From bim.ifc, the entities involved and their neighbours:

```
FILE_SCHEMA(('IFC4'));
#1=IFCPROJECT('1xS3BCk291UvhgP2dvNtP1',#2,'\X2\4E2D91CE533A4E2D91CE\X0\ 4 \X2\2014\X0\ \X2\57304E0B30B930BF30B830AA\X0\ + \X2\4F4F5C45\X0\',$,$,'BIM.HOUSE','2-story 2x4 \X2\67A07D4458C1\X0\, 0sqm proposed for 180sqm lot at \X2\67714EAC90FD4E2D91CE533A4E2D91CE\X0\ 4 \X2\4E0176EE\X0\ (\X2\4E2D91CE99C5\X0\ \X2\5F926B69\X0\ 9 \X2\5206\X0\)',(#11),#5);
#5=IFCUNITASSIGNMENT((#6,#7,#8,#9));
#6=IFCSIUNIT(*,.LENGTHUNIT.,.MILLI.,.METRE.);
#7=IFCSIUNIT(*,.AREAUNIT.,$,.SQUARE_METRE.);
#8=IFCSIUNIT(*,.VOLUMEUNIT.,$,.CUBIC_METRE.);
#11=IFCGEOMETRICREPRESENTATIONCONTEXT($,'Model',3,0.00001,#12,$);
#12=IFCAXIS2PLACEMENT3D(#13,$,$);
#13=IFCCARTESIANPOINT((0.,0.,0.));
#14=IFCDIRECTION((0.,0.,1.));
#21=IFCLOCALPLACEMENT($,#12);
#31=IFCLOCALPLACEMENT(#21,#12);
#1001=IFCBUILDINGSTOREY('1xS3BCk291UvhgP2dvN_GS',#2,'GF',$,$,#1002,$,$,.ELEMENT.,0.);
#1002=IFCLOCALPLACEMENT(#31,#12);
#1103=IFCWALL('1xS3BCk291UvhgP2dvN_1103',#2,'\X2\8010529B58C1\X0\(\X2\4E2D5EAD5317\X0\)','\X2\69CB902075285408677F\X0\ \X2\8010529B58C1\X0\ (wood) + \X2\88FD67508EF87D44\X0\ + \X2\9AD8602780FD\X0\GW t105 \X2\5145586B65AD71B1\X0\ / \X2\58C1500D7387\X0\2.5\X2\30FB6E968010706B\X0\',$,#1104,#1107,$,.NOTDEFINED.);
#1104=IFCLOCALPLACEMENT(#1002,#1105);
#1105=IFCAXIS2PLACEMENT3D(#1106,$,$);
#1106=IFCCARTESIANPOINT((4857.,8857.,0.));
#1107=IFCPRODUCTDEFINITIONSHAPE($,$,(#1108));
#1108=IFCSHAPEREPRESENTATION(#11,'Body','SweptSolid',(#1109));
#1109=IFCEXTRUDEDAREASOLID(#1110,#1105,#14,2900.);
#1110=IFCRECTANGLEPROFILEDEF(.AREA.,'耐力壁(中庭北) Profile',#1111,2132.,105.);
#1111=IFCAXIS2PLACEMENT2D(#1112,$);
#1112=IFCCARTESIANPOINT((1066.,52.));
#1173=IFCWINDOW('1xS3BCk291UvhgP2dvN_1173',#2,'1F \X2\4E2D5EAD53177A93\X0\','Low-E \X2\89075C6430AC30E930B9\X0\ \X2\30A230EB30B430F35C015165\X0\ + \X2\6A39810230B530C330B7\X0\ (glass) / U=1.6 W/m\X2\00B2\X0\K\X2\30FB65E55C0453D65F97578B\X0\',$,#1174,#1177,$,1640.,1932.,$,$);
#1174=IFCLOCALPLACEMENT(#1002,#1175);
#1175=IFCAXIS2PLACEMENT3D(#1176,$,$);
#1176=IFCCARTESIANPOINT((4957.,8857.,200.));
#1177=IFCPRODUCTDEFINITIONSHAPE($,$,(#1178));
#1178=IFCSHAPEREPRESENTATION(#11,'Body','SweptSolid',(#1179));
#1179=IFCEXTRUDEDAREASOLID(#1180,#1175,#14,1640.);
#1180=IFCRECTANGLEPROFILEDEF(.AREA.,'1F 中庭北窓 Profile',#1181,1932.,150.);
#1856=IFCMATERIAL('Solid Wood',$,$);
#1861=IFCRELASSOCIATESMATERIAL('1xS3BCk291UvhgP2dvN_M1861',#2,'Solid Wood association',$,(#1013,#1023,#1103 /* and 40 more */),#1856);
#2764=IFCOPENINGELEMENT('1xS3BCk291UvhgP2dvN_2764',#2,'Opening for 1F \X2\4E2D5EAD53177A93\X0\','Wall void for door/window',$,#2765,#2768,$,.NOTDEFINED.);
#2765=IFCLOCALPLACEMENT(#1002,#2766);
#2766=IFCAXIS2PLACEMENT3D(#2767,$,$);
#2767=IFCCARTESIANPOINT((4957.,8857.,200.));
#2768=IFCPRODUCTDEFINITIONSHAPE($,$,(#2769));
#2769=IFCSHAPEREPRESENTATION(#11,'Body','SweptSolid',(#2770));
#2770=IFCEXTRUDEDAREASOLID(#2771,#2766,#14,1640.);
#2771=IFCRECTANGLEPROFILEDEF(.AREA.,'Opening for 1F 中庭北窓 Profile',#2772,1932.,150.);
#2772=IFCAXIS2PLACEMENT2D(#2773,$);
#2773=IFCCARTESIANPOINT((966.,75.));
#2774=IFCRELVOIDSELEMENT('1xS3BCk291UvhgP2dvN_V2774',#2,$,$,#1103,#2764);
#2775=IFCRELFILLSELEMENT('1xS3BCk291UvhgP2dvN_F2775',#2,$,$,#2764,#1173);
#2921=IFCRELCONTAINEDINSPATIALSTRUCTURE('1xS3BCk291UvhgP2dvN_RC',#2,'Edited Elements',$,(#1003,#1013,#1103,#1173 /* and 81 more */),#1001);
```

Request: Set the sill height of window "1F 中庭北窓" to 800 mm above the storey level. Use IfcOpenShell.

```python
import numpy as np
import ifcopenshell
import ifcopenshell.api.geometry
import ifcopenshell.geom
import ifcopenshell.util.element
import ifcopenshell.util.placement
import ifcopenshell.util.shape
import ifcopenshell.util.unit

model = ifcopenshell.open("bim.ifc")
unit_scale = ifcopenshell.util.unit.calculate_unit_scale(model)

window = model.by_guid("1xS3BCk291UvhgP2dvN_1173")
opening = window.FillsVoids[0].RelatingOpeningElement
storey = ifcopenshell.util.element.get_container(window, ifc_class="IfcBuildingStorey")
level = ifcopenshell.util.placement.get_local_placement(storey.ObjectPlacement)[2, 3]

# The opening's origin need not be at the sill, so measure its lowest point.
shape = ifcopenshell.geom.create_shape(ifcopenshell.geom.settings(), opening)
bottom = ifcopenshell.util.shape.get_shape_bottom_elevation(shape, shape.geometry) / unit_scale
dz = level + 0.8 / unit_scale - bottom

shift = np.array([0.0, 0.0, dz])
# The window is not placed relative to its opening, so move both.
for product in (opening, window):
    matrix = ifcopenshell.util.placement.get_local_placement(product.ObjectPlacement)
    matrix[:3, 3] += shift
    ifcopenshell.api.geometry.edit_object_placement(model, product=product, matrix=matrix, is_si=False)

print(f"moved by {dz * unit_scale:+.3f} m")

model.write("bim_rev.ifc")
```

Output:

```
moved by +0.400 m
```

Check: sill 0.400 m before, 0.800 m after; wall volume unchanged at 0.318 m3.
